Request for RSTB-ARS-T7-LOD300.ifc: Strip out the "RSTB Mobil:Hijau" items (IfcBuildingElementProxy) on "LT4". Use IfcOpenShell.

First a look at what the model holds.

```python
import ifcopenshell
import ifcopenshell.util.element

model = ifcopenshell.open("RSTB-ARS-T7-LOD300.ifc")
print(model.schema)
storey = next(s for s in model.by_type("IfcBuildingStorey") if s.Name == "LT4")
proxies = [e for e in ifcopenshell.util.element.get_decomposition(storey) if e.is_a("IfcBuildingElementProxy")]
seen = {}
for e in proxies:
    element_type = ifcopenshell.util.element.get_type(e)
    name = element_type.Name if element_type not in (None, e) else None
    seen[name] = seen.get(name, 0) + 1
for name, count in sorted(seen.items(), key=str):
    print(count, "x", name)
```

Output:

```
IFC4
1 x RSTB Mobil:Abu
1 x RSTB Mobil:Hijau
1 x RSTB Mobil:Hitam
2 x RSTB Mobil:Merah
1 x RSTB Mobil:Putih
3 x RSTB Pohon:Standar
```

```python
import ifcopenshell
import ifcopenshell.api.root
import ifcopenshell.util.element

model = ifcopenshell.open("RSTB-ARS-T7-LOD300.ifc")

storey = next(s for s in model.by_type("IfcBuildingStorey") if s.Name == "LT4")
proxies = [e for e in ifcopenshell.util.element.get_decomposition(storey) if e.is_a("IfcBuildingElementProxy")]
targets = [e for e in proxies if (t := ifcopenshell.util.element.get_type(e)) not in (None, e) and t.Name == "RSTB Mobil:Hijau"]

for e in targets:
    ifcopenshell.api.root.remove_product(model, product=e)
print(len(targets), "removed")

model.write("RSTB-ARS-T7-LOD300_edited.ifc")
```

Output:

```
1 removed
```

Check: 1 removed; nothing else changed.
